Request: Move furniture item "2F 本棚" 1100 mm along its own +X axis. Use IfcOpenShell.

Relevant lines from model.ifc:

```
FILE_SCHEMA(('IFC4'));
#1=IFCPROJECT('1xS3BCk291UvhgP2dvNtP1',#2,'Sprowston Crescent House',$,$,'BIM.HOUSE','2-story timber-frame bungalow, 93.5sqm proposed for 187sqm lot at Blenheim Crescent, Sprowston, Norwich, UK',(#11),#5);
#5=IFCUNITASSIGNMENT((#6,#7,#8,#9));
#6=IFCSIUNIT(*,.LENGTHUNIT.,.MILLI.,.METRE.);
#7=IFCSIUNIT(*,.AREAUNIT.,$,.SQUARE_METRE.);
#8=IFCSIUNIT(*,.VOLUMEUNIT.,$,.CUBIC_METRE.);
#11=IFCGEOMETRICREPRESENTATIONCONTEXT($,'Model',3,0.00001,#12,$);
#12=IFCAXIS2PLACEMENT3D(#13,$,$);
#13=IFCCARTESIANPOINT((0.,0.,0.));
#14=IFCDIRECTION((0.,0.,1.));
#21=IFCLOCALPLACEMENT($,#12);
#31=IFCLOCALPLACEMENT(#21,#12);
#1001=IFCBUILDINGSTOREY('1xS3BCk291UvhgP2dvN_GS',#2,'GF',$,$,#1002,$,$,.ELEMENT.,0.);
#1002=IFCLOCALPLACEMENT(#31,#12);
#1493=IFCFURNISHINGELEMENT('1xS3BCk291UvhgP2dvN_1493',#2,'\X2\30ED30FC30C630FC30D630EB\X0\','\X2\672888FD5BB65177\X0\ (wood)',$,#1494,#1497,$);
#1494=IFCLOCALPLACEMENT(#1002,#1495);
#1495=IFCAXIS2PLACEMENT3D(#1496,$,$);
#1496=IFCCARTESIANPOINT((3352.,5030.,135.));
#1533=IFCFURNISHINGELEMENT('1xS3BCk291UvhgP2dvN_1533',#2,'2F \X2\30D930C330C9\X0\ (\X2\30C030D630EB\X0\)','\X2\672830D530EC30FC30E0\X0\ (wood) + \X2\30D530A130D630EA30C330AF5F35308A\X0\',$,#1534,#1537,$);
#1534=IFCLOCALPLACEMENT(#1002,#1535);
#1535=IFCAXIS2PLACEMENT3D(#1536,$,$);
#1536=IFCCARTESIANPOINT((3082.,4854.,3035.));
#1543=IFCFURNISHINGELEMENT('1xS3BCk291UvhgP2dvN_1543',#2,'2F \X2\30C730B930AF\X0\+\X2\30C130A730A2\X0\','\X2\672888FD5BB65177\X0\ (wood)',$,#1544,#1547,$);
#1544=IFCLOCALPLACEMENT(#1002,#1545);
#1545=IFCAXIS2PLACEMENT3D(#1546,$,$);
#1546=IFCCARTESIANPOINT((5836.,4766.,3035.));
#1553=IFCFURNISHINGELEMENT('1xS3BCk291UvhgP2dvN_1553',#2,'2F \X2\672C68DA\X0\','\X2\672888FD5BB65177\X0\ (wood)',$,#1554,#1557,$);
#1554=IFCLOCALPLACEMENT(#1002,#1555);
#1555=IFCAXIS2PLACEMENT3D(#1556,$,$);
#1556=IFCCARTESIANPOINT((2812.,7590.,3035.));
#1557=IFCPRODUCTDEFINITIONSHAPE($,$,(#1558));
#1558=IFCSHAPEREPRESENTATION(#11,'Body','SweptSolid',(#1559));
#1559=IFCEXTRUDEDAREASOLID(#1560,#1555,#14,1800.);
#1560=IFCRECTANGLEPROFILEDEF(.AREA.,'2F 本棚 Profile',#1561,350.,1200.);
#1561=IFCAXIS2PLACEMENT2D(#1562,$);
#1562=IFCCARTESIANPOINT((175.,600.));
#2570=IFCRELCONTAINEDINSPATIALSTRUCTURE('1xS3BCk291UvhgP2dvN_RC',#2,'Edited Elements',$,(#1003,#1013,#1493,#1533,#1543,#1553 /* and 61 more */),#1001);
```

```python
import ifcopenshell
import ifcopenshell.api.geometry
import ifcopenshell.util.placement

model = ifcopenshell.open("model.ifc")

item = model.by_id(1553)
matrix = ifcopenshell.util.placement.get_local_placement(item.ObjectPlacement)
matrix[:3, 3] += matrix[:3, 0] * 1100.0
ifcopenshell.api.geometry.edit_object_placement(model, product=item, matrix=matrix, is_si=False)

print(ifcopenshell.util.placement.get_local_placement(item.ObjectPlacement).round(3) + 0.0)

model.write("model_edited.ifc")
```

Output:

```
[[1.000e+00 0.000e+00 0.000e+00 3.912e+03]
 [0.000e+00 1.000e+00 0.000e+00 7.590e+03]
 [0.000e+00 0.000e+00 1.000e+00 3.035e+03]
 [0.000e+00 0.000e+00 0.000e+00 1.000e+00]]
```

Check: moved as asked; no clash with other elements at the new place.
